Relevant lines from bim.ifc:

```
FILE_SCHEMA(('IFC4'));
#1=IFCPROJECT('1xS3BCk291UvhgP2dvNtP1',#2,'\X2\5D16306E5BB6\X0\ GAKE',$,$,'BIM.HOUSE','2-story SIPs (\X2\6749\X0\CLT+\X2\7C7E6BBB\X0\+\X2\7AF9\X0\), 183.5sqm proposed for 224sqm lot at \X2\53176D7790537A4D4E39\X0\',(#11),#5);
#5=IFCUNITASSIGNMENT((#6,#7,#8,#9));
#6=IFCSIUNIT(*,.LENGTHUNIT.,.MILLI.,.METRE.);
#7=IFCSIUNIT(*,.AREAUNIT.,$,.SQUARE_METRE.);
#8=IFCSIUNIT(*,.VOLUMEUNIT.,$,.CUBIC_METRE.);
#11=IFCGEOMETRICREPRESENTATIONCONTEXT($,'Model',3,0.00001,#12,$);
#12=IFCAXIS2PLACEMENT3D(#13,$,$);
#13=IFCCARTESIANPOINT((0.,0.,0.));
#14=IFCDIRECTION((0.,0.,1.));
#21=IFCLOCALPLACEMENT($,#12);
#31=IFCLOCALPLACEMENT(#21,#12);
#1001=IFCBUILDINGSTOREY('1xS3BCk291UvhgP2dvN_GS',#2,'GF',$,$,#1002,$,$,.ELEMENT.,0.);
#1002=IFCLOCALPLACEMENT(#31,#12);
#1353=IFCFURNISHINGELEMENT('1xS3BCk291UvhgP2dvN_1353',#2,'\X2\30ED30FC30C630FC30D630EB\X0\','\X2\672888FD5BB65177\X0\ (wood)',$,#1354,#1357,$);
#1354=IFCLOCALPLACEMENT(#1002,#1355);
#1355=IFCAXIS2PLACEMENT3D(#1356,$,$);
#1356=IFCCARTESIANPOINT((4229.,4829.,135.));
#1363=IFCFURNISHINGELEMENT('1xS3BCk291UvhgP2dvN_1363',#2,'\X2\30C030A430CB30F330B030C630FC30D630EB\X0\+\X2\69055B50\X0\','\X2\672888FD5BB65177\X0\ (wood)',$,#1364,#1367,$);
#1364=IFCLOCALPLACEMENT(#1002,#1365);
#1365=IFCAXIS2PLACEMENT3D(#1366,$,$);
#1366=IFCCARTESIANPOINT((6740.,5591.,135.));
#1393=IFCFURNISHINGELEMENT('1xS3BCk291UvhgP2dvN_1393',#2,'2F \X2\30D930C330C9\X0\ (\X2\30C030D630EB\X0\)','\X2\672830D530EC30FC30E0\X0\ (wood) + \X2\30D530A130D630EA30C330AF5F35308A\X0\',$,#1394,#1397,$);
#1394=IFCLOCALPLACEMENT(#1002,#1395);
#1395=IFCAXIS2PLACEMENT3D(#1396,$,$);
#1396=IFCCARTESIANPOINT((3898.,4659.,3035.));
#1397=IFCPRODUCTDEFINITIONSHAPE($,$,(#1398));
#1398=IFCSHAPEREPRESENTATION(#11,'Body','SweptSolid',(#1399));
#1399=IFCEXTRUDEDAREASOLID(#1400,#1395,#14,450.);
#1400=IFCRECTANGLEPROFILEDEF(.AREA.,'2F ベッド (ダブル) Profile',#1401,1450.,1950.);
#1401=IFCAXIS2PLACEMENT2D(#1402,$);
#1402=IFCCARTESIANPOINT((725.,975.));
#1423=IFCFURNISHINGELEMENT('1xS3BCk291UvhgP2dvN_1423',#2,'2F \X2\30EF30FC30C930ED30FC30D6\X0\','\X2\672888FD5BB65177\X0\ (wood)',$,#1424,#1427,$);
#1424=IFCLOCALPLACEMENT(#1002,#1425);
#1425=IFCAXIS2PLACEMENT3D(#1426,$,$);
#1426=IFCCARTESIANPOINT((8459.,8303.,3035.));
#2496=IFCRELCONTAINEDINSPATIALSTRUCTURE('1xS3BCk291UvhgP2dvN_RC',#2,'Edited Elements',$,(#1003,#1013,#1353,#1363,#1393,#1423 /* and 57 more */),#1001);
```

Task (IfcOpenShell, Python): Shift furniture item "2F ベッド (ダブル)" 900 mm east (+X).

```python
import ifcopenshell
import ifcopenshell.api.geometry
import ifcopenshell.util.placement
import ifcopenshell.util.unit

model = ifcopenshell.open("bim.ifc")
unit_scale = ifcopenshell.util.unit.calculate_unit_scale(model)

item = model.by_id(1393)
matrix = ifcopenshell.util.placement.get_local_placement(item.ObjectPlacement)
matrix[0, 3] += 0.9 / unit_scale
ifcopenshell.api.geometry.edit_object_placement(model, product=item, matrix=matrix, is_si=False)

print(ifcopenshell.util.placement.get_local_placement(item.ObjectPlacement).round(3) + 0.0)

model.write("bim_rev.ifc")
```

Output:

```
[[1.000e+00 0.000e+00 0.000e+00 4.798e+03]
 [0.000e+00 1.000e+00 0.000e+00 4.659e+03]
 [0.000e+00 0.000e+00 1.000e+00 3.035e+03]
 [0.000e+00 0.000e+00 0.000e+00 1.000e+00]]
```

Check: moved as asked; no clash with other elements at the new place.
